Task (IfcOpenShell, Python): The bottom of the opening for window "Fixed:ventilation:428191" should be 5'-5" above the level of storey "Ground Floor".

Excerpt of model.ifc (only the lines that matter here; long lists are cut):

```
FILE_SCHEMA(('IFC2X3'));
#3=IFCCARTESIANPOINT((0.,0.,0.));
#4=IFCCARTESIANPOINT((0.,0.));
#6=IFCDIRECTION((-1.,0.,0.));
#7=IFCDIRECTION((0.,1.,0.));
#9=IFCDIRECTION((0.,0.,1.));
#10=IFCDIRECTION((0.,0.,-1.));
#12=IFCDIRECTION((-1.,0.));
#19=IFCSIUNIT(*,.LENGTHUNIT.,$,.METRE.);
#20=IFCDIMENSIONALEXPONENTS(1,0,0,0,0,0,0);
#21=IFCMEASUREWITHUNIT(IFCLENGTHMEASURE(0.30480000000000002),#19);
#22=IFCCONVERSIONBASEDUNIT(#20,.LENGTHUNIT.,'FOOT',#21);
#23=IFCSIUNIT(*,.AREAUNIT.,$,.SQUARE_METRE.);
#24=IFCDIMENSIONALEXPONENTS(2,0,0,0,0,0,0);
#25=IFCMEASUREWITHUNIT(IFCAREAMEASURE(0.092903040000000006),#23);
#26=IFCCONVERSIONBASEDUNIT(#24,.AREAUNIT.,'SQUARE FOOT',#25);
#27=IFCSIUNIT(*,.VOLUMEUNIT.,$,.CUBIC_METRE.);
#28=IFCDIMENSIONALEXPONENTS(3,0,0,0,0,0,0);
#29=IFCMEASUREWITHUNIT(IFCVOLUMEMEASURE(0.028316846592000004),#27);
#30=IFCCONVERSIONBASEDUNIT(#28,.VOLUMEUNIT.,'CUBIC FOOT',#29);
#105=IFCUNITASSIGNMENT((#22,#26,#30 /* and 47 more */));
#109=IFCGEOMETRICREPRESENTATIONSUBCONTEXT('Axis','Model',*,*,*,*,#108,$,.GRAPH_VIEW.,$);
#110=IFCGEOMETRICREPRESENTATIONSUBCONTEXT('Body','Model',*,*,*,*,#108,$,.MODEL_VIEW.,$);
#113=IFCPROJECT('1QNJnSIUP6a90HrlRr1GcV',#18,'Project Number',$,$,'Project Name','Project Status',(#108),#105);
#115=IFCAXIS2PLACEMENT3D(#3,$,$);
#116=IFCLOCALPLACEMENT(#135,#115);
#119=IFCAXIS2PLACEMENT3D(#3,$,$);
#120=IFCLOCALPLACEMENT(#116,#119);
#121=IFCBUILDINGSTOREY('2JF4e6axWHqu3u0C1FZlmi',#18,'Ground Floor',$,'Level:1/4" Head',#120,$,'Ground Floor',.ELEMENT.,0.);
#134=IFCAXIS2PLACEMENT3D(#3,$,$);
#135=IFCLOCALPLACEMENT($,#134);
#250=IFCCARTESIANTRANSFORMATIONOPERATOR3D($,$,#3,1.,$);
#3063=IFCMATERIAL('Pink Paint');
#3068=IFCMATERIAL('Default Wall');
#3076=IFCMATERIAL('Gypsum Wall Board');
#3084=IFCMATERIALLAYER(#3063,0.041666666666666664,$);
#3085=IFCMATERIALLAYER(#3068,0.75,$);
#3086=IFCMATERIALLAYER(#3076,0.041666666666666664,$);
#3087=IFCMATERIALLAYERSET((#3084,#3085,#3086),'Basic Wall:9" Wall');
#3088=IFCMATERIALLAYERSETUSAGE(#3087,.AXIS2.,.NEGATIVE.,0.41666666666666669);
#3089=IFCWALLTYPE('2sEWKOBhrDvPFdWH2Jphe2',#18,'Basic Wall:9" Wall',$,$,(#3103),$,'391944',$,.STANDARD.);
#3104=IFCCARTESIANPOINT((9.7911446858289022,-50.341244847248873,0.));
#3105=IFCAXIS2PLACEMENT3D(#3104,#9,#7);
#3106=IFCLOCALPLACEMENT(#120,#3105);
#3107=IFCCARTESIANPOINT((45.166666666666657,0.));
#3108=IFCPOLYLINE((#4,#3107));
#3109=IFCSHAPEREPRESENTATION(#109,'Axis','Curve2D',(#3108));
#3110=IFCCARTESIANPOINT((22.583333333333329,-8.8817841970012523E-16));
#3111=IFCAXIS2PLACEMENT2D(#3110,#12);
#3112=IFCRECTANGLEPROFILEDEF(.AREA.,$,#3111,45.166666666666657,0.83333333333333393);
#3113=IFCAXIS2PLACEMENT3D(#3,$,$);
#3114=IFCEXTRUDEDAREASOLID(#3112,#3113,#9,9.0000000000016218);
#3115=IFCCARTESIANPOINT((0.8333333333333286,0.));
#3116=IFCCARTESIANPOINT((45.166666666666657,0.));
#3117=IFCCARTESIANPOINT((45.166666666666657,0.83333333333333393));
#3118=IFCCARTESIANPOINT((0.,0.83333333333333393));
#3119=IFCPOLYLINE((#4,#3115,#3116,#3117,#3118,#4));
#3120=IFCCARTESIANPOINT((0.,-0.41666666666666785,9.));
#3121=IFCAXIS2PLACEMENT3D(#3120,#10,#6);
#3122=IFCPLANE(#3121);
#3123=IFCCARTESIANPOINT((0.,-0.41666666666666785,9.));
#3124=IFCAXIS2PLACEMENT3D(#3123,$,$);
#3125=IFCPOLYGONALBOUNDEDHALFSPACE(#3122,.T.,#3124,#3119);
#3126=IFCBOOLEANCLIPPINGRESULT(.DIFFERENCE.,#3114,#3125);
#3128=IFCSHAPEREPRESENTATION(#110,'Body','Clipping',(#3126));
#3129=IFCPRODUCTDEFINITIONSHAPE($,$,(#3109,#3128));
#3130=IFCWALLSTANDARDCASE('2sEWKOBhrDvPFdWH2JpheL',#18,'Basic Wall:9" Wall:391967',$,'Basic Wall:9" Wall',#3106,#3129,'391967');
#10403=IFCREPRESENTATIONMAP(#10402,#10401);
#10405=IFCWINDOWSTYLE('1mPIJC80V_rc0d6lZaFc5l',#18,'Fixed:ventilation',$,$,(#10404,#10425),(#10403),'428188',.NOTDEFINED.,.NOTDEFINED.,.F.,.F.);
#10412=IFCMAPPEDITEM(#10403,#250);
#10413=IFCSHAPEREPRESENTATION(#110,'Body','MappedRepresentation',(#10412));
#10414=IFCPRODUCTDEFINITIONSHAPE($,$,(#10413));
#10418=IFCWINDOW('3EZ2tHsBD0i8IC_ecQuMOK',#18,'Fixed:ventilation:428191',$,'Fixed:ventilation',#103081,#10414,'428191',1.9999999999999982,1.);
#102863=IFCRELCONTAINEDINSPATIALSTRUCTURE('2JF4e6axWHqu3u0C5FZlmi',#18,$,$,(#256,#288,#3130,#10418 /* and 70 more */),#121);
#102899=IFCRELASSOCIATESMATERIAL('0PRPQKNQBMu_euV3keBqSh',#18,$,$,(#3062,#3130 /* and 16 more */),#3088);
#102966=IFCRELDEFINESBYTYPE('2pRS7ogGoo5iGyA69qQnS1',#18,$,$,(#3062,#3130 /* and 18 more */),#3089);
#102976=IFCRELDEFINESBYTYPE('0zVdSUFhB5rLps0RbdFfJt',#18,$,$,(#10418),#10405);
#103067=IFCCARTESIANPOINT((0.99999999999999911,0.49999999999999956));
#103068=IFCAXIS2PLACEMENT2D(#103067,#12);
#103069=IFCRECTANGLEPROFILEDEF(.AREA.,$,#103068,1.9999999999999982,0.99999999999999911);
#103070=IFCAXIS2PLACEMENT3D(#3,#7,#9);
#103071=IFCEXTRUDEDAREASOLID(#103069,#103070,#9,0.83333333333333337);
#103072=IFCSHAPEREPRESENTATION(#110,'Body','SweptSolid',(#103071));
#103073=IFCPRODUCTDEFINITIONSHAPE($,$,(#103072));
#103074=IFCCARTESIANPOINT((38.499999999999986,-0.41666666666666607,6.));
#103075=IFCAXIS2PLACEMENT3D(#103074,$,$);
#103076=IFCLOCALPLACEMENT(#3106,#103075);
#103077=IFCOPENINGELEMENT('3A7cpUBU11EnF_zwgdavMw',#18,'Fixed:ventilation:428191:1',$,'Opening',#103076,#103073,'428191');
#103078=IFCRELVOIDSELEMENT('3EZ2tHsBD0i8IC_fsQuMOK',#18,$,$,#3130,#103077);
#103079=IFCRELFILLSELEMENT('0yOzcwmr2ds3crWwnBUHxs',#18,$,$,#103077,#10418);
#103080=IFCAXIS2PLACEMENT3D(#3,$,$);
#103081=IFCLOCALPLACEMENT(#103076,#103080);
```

```python
import numpy as np
import ifcopenshell
import ifcopenshell.api.geometry
import ifcopenshell.geom
import ifcopenshell.util.element
import ifcopenshell.util.placement
import ifcopenshell.util.shape
import ifcopenshell.util.unit

model = ifcopenshell.open("model.ifc")
unit_scale = ifcopenshell.util.unit.calculate_unit_scale(model)

window = model.by_guid("3EZ2tHsBD0i8IC_ecQuMOK")
opening = window.FillsVoids[0].RelatingOpeningElement
storey = ifcopenshell.util.element.get_container(window, ifc_class="IfcBuildingStorey")
level = ifcopenshell.util.placement.get_local_placement(storey.ObjectPlacement)[2, 3]

# The opening's origin need not be at the sill, so measure its lowest point.
shape = ifcopenshell.geom.create_shape(ifcopenshell.geom.settings(), opening)
bottom = ifcopenshell.util.shape.get_shape_bottom_elevation(shape, shape.geometry) / unit_scale
dz = level + 65 * 0.0254 / unit_scale - bottom

shift = np.array([0.0, 0.0, dz])
# The window is placed relative to its opening, so it follows when the opening moves.
matrix = ifcopenshell.util.placement.get_local_placement(opening.ObjectPlacement)
matrix[:3, 3] += shift
ifcopenshell.api.geometry.edit_object_placement(
    model, product=opening, matrix=matrix, is_si=False, should_transform_children=True
)

print(f"moved by {dz * unit_scale:+.3f} m")

model.write("model_updated.ifc")
```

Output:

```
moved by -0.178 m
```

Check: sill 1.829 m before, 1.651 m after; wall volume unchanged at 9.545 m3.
